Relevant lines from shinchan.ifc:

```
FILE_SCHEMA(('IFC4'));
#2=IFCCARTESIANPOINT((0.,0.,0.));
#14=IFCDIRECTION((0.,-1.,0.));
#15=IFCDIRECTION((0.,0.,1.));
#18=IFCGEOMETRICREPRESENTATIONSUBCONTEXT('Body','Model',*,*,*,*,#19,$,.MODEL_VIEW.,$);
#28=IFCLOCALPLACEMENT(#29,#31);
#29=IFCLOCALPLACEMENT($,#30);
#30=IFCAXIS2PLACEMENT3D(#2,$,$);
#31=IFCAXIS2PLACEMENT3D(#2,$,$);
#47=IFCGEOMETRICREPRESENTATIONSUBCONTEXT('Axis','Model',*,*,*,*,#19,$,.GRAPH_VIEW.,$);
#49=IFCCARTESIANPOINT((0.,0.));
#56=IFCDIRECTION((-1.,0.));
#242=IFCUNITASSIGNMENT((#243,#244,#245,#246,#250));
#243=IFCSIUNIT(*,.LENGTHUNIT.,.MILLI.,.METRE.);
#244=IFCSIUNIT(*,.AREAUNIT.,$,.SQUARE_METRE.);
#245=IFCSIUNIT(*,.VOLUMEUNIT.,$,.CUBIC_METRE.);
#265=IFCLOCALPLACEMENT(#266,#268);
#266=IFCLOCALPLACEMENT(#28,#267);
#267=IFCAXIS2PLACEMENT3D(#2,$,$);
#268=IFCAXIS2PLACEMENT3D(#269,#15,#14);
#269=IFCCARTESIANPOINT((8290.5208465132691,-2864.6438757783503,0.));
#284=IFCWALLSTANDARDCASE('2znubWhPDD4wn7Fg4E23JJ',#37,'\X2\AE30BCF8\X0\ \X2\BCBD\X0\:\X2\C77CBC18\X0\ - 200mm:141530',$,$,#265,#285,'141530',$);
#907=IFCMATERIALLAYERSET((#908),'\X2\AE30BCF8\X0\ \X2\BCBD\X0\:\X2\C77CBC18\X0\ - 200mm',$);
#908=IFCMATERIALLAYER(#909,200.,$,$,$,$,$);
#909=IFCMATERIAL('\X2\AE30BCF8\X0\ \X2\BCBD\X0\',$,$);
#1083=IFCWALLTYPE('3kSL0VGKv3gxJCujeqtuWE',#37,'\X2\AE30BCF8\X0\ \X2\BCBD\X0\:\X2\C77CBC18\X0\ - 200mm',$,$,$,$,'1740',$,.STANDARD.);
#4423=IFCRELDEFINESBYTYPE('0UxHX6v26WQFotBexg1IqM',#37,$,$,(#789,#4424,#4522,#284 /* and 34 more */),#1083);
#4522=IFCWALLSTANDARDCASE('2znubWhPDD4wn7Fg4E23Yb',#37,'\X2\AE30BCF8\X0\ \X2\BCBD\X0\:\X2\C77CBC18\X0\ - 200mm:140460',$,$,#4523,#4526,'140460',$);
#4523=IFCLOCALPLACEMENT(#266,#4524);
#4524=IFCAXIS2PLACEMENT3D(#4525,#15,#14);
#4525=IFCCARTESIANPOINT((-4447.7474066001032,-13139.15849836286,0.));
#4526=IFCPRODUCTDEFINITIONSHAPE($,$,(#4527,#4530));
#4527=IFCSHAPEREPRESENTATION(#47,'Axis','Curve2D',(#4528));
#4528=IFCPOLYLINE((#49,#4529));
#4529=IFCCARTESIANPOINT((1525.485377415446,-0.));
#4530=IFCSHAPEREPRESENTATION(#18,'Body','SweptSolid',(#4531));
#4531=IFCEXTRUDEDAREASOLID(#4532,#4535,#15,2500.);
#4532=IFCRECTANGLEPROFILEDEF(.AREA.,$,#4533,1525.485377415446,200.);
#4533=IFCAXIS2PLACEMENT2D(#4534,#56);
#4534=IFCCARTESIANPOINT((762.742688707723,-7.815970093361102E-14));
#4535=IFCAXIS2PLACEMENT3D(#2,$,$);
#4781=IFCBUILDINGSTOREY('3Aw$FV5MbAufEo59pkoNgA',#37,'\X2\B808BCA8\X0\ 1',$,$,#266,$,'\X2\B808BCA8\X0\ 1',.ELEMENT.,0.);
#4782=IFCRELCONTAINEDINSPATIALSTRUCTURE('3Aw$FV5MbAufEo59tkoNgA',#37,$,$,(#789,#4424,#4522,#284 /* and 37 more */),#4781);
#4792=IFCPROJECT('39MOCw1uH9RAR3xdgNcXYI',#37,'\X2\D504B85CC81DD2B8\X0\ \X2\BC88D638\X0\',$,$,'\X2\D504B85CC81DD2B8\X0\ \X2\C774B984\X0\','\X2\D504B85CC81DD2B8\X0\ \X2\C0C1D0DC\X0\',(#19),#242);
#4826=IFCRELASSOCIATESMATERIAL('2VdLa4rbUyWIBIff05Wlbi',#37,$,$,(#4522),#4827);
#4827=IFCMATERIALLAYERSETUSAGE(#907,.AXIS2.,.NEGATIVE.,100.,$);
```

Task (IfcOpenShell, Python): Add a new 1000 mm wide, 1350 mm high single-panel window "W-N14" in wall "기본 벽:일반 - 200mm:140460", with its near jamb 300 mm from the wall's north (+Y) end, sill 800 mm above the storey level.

```python
import numpy as np
import ifcopenshell
import ifcopenshell.api.feature
import ifcopenshell.api.geometry
import ifcopenshell.api.root
import ifcopenshell.api.spatial
import ifcopenshell.geom
import ifcopenshell.util.element
import ifcopenshell.util.placement
import ifcopenshell.util.representation
import ifcopenshell.util.shape
import ifcopenshell.util.unit

model = ifcopenshell.open("shinchan.ifc")
unit_scale = ifcopenshell.util.unit.calculate_unit_scale(model)
settings = ifcopenshell.geom.settings()


def volume(element):
    """Net volume in cubic metres, openings subtracted."""
    shape = ifcopenshell.geom.create_shape(settings, element)
    return ifcopenshell.util.shape.get_volume(shape.geometry)


wall = model.by_id(4522)
storey = ifcopenshell.util.element.get_container(wall, ifc_class="IfcBuildingStorey")
context = ifcopenshell.util.representation.get_context(model, "Model", "Body", "MODEL_VIEW")
before = volume(wall)

width, height, from_end, sill = 1, 1.35, 0.3, 0.8  # metres

# The wall runs along its own X axis, and the end named is its -X end.
wall_shape = ifcopenshell.geom.create_shape(settings, wall)
x, y, z = ifcopenshell.util.shape.get_vertices(wall_shape.geometry).T
start = x.min() + from_end
face, thickness = float(y.min()), float(y.max() - y.min())
wall_matrix = ifcopenshell.util.placement.get_local_placement(wall.ObjectPlacement)
level = ifcopenshell.util.placement.get_local_placement(storey.ObjectPlacement)[2, 3]


def in_wall(x, y):
    """Placement at x, y metres in the wall's axes, at sill height."""
    matrix = wall_matrix.copy()
    matrix[:, 3] = wall_matrix @ np.array([x / unit_scale, y / unit_scale, 0.0, 1.0])
    matrix[2, 3] = level + sill / unit_scale
    return matrix


# Opening: a box that overshoots both wall faces by 50 mm.
opening = ifcopenshell.api.root.create_entity(model, ifc_class="IfcOpeningElement", predefined_type="OPENING")
box = ifcopenshell.api.geometry.add_wall_representation(
    model, context=context, length=width, height=height, thickness=thickness + 0.1
)
ifcopenshell.api.geometry.assign_representation(model, product=opening, representation=box)
ifcopenshell.api.geometry.edit_object_placement(model, product=opening, matrix=in_wall(start, face - 0.05), is_si=False)
ifcopenshell.api.feature.add_feature(model, feature=opening, element=wall)

window = ifcopenshell.api.root.create_entity(model, ifc_class="IfcWindow", name="W-N14", predefined_type="WINDOW")
window.OverallWidth, window.OverallHeight = width / unit_scale, height / unit_scale
window.PartitioningType = "SINGLE_PANEL"
body = ifcopenshell.api.geometry.add_window_representation(
    model,
    context=context,
    overall_width=window.OverallWidth,
    overall_height=window.OverallHeight,
    partition_type="SINGLE_PANEL",
)
ifcopenshell.api.geometry.assign_representation(model, product=window, representation=body)
ifcopenshell.api.spatial.assign_container(model, products=[window], relating_structure=storey)
ifcopenshell.api.feature.add_filling(model, opening=opening, element=window)

# Centre the window in the wall's thickness.
ifcopenshell.api.geometry.edit_object_placement(model, product=window, matrix=in_wall(start, face), is_si=False)
window_shape = ifcopenshell.geom.create_shape(settings, window)
depth = ifcopenshell.util.shape.get_vertices(window_shape.geometry)[:, 1]
offset = face + thickness / 2 - (depth.min() + depth.max()) / 2
ifcopenshell.api.geometry.edit_object_placement(model, product=window, matrix=in_wall(start, offset), is_si=False)

after = volume(wall)

print(f"wall volume {before:.3f} -> {after:.3f} m3")

model.write("shinchan_edited.ifc")
```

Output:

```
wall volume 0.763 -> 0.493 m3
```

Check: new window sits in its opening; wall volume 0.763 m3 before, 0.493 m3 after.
